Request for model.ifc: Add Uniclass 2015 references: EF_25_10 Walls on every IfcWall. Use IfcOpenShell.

First a look at what the model holds.

```python
import ifcopenshell

model = ifcopenshell.open("model.ifc")
print(model.schema)
print("classifications:", [c.Name for c in model.by_type("IfcClassification")])
for ifc_class in ("IfcDoor", "IfcRoof", "IfcStair", "IfcWall", "IfcWindow"):
    print(ifc_class, len(model.by_type(ifc_class)))
```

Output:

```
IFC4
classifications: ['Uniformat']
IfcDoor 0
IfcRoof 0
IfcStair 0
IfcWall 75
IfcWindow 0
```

```python
import ifcopenshell
import ifcopenshell.api.classification

model = ifcopenshell.open("model.ifc")

system = ifcopenshell.api.classification.add_classification(model, classification="Uniclass 2015")

codes = {
    "IfcWall": ("EF_25_10", "Walls"),
}
for ifc_class, (code, name) in codes.items():
    products = model.by_type(ifc_class)
    ifcopenshell.api.classification.add_reference(
        model, products=products, classification=system, identification=code, name=name
    )
    print(code, len(products))

model.write("model_rev.ifc")
```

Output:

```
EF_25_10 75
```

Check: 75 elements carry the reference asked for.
